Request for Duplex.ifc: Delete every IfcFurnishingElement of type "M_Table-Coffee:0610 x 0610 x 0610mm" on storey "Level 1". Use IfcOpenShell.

First a look at what the model holds.

```python
import ifcopenshell
import ifcopenshell.util.element

model = ifcopenshell.open("Duplex.ifc")
print(model.schema)
storey = next(s for s in model.by_type("IfcBuildingStorey") if s.Name == "Level 1")
furniture = [e for e in ifcopenshell.util.element.get_decomposition(storey) if e.is_a("IfcFurnishingElement")]
seen = {}
for e in furniture:
    element_type = ifcopenshell.util.element.get_type(e)
    name = element_type.Name if element_type not in (None, e) else None
    seen[name] = seen.get(name, 0) + 1
for name, count in sorted(seen.items(), key=str):
    print(count, "x", name)
```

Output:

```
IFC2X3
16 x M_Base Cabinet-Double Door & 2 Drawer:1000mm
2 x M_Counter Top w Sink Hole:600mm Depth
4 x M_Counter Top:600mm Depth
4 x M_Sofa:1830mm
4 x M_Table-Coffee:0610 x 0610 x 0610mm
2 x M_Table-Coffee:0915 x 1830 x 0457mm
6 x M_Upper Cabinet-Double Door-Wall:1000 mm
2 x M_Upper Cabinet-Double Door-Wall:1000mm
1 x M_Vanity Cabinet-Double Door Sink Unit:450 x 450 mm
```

```python
import ifcopenshell
import ifcopenshell.api.root
import ifcopenshell.util.element

model = ifcopenshell.open("Duplex.ifc")

storey = next(s for s in model.by_type("IfcBuildingStorey") if s.Name == "Level 1")
furniture = [e for e in ifcopenshell.util.element.get_decomposition(storey) if e.is_a("IfcFurnishingElement")]
targets = [e for e in furniture if (t := ifcopenshell.util.element.get_type(e)) not in (None, e) and t.Name == "M_Table-Coffee:0610 x 0610 x 0610mm"]

for e in targets:
    ifcopenshell.api.root.remove_product(model, product=e)
print(len(targets), "removed")

model.write("Duplex_edited.ifc")
```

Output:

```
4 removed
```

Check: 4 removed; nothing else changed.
